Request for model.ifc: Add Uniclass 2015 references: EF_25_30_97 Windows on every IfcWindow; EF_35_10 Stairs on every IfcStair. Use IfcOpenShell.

First a look at what the model holds.

```python
import ifcopenshell

model = ifcopenshell.open("model.ifc")
print(model.schema)
print("classifications:", [c.Name for c in model.by_type("IfcClassification")])
for ifc_class in ("IfcDoor", "IfcRoof", "IfcStair", "IfcWall", "IfcWindow"):
    print(ifc_class, len(model.by_type(ifc_class)))
```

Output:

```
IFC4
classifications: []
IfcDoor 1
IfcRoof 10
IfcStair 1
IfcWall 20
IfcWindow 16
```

```python
import ifcopenshell
import ifcopenshell.api.classification

model = ifcopenshell.open("model.ifc")

system = ifcopenshell.api.classification.add_classification(model, classification="Uniclass 2015")

codes = {
    "IfcWindow": ("EF_25_30_97", "Windows"),
    "IfcStair": ("EF_35_10", "Stairs"),
}
for ifc_class, (code, name) in codes.items():
    products = model.by_type(ifc_class)
    ifcopenshell.api.classification.add_reference(
        model, products=products, classification=system, identification=code, name=name
    )
    print(code, len(products))

model.write("model_rev.ifc")
```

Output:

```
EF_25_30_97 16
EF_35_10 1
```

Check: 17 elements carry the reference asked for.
